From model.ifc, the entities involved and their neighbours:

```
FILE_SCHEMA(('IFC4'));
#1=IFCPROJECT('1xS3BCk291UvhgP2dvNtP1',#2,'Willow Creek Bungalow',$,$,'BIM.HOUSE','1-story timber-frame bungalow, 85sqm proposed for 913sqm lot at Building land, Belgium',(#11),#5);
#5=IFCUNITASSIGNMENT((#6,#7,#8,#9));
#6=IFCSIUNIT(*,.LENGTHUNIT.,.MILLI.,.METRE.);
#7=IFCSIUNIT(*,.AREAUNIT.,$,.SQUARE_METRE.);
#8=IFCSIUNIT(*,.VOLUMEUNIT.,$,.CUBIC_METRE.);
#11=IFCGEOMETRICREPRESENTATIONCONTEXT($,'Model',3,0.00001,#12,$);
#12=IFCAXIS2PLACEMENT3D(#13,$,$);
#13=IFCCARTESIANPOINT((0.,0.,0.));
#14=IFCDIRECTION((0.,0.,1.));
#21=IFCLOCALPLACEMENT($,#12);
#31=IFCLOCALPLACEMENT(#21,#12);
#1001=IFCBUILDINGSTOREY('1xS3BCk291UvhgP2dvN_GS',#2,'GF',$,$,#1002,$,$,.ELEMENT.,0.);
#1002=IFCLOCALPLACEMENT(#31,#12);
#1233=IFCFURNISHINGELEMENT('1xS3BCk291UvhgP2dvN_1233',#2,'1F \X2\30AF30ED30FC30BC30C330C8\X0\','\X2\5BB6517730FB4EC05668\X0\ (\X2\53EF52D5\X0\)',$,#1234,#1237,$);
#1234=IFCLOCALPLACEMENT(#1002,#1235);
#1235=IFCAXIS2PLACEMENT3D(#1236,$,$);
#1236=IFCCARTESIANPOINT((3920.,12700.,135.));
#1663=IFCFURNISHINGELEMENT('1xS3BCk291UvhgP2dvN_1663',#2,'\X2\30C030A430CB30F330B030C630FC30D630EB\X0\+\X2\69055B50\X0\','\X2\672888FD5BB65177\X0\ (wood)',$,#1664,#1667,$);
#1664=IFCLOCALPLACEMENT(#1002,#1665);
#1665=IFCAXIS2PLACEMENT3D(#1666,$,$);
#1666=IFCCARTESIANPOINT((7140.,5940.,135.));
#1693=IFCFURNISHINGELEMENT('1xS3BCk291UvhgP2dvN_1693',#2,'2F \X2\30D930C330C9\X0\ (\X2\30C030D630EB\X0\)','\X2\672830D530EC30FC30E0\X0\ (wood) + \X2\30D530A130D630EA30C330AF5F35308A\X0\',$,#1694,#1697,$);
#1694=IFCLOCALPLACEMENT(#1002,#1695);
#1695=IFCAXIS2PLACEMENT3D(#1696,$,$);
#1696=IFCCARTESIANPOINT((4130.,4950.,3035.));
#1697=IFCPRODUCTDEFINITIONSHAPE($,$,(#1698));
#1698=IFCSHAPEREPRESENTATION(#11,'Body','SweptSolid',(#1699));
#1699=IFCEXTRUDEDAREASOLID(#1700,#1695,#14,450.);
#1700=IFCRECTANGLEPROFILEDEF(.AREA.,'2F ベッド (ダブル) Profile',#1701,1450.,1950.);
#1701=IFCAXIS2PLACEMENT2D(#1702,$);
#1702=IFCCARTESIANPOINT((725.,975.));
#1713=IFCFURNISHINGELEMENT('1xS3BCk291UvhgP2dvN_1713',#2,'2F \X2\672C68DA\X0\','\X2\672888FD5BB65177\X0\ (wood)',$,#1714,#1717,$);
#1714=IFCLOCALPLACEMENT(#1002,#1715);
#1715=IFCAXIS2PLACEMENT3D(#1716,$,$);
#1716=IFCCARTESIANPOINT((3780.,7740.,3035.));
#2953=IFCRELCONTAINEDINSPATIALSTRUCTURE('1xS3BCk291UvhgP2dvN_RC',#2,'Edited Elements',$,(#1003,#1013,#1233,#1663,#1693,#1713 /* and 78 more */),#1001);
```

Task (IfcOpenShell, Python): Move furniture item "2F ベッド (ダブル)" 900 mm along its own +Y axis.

```python
import ifcopenshell
import ifcopenshell.api.geometry
import ifcopenshell.util.placement
import ifcopenshell.util.unit

model = ifcopenshell.open("model.ifc")
unit_scale = ifcopenshell.util.unit.calculate_unit_scale(model)

item = model.by_id(1693)
matrix = ifcopenshell.util.placement.get_local_placement(item.ObjectPlacement)
matrix[:3, 3] += matrix[:3, 1] * 0.9 / unit_scale
ifcopenshell.api.geometry.edit_object_placement(model, product=item, matrix=matrix, is_si=False)

print(ifcopenshell.util.placement.get_local_placement(item.ObjectPlacement).round(3) + 0.0)

model.write("model_v2.ifc")
```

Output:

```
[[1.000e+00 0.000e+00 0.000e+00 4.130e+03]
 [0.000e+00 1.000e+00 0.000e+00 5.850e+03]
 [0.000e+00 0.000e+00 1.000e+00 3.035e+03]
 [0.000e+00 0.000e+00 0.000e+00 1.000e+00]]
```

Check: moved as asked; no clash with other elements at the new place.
